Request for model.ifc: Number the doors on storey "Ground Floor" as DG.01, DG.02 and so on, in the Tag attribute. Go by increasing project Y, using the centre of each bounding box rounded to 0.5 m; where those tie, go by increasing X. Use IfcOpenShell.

First a look at what the model holds.

```python
import ifcopenshell
import ifcopenshell.util.element
import ifcopenshell.util.placement

model = ifcopenshell.open("model.ifc")
print(model.schema)
storey = next(s for s in model.by_type("IfcBuildingStorey") if s.Name == "Ground Floor")
doors = [e for e in ifcopenshell.util.element.get_decomposition(storey) if e.is_a("IfcDoor")]
for e in sorted(doors, key=lambda e: e.id()):
    origin = ifcopenshell.util.placement.get_local_placement(e.ObjectPlacement)[:3, 3]
    print(e.id(), e.Tag, e.Name, origin.round(2) + 0.0, sep=" | ")
```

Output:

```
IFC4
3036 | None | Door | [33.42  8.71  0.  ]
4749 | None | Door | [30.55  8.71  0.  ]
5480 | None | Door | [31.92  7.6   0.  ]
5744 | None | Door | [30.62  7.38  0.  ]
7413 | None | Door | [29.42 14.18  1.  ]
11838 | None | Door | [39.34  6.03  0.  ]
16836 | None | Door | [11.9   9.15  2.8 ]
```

```python
import ifcopenshell
import ifcopenshell.geom
import ifcopenshell.util.element
import ifcopenshell.util.shape

model = ifcopenshell.open("model.ifc")
settings = ifcopenshell.geom.settings()
settings.set("use-world-coords", True)


def centre(element):
    shape = ifcopenshell.geom.create_shape(settings, element)
    return ifcopenshell.util.shape.get_bbox_centroid(shape.geometry)


storey = next(s for s in model.by_type("IfcBuildingStorey") if s.Name == "Ground Floor")
doors = [e for e in ifcopenshell.util.element.get_decomposition(storey) if e.is_a("IfcDoor")]

# Insertion points can sit at a corner or the storey origin, so sort by the geometry (in metres).
centres = {e: centre(e) for e in doors}
doors.sort(key=lambda e: (round(centres[e][1] / 0.5), centres[e][0]))

for i, e in enumerate(doors, start=1):
    number = f"DG.{i:02d}"
    e.Tag = number
    print(e.id(), number)

model.write("model_rev.ifc")
```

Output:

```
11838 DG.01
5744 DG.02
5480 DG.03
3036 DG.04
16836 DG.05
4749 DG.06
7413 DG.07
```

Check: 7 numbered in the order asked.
